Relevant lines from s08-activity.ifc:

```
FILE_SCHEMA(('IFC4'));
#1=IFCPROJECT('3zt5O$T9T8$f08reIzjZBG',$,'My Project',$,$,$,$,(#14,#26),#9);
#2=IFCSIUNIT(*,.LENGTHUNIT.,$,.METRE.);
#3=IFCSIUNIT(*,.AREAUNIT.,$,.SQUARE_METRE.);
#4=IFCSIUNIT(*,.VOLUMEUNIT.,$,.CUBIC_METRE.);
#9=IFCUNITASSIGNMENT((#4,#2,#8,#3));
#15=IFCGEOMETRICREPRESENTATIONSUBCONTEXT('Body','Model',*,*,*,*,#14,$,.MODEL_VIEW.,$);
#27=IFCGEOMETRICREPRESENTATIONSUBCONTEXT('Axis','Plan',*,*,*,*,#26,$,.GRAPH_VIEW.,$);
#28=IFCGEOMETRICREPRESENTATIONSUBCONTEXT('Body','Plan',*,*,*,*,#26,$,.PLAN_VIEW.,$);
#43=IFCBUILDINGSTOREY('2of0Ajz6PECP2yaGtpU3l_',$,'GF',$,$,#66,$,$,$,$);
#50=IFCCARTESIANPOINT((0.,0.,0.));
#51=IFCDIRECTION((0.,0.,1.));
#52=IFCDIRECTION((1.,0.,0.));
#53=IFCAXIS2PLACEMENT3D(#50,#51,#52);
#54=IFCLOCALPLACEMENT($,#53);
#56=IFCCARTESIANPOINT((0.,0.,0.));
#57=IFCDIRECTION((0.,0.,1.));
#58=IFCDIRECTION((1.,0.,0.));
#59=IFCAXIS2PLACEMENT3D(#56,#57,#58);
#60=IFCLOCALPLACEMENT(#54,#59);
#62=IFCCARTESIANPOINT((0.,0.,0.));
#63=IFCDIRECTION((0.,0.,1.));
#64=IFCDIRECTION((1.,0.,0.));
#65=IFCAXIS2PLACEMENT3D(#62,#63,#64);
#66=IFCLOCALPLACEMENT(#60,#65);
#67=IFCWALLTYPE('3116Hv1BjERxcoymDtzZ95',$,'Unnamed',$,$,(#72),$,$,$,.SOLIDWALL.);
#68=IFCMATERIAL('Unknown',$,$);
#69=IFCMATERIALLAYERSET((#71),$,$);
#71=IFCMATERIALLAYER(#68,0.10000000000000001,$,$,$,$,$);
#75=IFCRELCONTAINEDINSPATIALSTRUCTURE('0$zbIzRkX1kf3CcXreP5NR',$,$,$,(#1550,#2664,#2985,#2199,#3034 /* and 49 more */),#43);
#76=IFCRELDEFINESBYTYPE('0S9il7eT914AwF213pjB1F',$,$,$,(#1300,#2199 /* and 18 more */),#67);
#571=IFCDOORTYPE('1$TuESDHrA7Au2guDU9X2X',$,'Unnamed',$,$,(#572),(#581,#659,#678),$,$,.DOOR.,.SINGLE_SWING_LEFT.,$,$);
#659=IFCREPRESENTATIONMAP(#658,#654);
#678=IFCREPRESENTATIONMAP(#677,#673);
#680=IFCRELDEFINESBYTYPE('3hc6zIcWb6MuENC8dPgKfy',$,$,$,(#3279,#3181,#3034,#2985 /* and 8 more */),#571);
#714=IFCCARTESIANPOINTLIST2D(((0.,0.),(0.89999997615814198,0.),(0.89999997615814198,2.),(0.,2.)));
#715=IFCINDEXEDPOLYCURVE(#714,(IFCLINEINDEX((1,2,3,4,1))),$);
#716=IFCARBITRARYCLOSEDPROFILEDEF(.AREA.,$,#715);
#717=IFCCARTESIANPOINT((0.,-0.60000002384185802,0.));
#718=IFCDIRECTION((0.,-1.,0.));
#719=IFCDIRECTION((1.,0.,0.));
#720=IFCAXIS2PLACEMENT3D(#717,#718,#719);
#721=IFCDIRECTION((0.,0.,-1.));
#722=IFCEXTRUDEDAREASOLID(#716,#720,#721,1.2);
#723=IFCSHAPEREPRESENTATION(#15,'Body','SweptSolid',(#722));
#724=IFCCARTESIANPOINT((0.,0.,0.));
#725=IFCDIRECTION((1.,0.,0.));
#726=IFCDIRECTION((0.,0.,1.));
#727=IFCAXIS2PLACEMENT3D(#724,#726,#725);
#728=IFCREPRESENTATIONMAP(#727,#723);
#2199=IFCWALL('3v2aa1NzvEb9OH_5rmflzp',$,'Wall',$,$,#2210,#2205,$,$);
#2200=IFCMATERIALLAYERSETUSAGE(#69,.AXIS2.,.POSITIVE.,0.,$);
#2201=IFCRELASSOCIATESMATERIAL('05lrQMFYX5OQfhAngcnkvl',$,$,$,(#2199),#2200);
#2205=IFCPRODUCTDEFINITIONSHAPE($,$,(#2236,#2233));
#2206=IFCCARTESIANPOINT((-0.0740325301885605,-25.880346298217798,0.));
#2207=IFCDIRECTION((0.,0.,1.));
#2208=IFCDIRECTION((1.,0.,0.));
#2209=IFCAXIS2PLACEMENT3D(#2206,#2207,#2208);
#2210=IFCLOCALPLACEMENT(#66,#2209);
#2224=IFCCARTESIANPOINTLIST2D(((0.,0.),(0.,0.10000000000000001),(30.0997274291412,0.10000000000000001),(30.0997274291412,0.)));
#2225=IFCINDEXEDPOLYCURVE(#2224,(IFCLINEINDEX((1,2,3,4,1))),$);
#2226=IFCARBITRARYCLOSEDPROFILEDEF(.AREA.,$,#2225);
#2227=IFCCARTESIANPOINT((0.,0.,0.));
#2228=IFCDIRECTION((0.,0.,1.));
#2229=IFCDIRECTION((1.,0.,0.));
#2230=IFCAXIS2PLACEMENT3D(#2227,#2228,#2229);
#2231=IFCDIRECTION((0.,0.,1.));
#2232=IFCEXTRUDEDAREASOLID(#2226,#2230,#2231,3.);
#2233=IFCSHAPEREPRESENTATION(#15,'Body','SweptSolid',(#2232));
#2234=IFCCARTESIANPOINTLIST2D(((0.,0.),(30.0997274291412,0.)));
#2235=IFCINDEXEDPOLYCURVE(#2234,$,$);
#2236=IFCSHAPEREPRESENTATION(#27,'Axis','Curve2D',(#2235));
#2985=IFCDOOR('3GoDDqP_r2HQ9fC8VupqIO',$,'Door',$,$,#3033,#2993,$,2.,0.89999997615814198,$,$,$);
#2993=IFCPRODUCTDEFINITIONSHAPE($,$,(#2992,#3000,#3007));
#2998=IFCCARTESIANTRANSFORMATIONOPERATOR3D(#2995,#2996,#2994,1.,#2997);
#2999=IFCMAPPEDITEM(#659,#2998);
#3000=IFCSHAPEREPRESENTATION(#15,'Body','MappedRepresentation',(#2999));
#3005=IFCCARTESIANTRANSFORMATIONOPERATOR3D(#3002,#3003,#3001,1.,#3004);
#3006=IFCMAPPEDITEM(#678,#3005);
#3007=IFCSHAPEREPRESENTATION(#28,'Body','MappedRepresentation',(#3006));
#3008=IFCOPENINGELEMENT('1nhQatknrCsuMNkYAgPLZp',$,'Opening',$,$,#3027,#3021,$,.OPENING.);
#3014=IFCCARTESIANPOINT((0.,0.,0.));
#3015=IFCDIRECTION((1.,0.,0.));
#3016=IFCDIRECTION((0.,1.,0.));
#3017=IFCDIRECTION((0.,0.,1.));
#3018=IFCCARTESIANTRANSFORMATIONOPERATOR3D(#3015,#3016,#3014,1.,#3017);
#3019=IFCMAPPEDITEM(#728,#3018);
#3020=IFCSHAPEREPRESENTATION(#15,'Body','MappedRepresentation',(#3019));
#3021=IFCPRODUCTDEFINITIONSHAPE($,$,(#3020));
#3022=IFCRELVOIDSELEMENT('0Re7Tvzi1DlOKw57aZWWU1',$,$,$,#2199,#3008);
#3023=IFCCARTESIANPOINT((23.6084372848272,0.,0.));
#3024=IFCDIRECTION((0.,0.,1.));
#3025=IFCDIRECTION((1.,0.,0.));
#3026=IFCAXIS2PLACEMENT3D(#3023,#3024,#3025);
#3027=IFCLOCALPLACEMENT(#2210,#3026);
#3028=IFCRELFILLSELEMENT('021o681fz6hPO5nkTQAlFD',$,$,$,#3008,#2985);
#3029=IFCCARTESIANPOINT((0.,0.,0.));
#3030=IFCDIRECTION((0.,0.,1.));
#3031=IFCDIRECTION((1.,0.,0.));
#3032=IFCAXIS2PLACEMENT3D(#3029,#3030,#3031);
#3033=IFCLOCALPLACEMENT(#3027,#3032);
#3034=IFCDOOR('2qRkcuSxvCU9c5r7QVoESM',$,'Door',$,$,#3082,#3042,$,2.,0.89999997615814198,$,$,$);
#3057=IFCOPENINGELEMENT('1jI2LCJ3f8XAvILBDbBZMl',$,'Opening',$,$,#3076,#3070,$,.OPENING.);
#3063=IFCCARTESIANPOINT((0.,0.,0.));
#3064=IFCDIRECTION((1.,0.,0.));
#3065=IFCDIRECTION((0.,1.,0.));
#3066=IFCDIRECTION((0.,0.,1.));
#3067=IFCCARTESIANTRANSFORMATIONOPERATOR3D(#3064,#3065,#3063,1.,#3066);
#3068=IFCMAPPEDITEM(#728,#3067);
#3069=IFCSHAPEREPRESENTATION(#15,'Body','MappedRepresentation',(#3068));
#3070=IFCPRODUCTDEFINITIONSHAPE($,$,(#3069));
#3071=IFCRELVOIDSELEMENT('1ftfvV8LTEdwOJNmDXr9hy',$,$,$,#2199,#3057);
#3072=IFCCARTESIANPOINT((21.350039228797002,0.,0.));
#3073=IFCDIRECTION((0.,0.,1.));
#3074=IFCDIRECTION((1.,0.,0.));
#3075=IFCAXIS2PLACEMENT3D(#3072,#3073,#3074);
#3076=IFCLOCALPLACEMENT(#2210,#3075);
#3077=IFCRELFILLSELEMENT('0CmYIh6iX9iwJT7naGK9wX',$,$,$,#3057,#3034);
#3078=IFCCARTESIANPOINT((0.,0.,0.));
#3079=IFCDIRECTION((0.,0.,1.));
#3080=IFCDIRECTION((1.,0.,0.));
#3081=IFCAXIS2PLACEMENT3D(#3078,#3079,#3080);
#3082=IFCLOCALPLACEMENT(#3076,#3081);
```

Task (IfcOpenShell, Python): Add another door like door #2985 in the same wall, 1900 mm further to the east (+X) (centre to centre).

```python
import ifcopenshell
import ifcopenshell.api.feature
import ifcopenshell.api.geometry
import ifcopenshell.api.root
import ifcopenshell.geom
import ifcopenshell.util.element
import ifcopenshell.util.placement
import ifcopenshell.util.shape
import ifcopenshell.util.unit

model = ifcopenshell.open("s08-activity.ifc")
unit_scale = ifcopenshell.util.unit.calculate_unit_scale(model)
settings = ifcopenshell.geom.settings()


def volume(element):
    """Net volume in cubic metres, openings subtracted."""
    shape = ifcopenshell.geom.create_shape(settings, element)
    return ifcopenshell.util.shape.get_volume(shape.geometry)


door = model.by_guid("3GoDDqP_r2HQ9fC8VupqIO")
opening = door.FillsVoids[0].RelatingOpeningElement
wall = opening.VoidsElements[0].RelatingBuildingElement
before = volume(wall)
shift = ifcopenshell.util.placement.get_local_placement(wall.ObjectPlacement)[:3, 0] * 1.9 / unit_scale

# copy_class copies the void relationship, type, container and properties, but no geometry.
new_opening = ifcopenshell.api.root.copy_class(model, product=opening)
new_opening.Representation = ifcopenshell.util.element.copy_deep(
    model, opening.Representation, exclude=["IfcGeometricRepresentationContext", "IfcRepresentationMap"]
)
new_door = ifcopenshell.api.root.copy_class(model, product=door)
new_door.Representation = ifcopenshell.util.element.copy_deep(
    model, door.Representation, exclude=["IfcGeometricRepresentationContext", "IfcRepresentationMap"]
)
ifcopenshell.api.feature.add_filling(model, opening=new_opening, element=new_door)

for old, new in ((opening, new_opening), (door, new_door)):
    matrix = ifcopenshell.util.placement.get_local_placement(old.ObjectPlacement)
    matrix[:3, 3] += shift
    ifcopenshell.api.geometry.edit_object_placement(model, product=new, matrix=matrix, is_si=False)

after = volume(wall)

print(f"wall volume {before:.3f} -> {after:.3f} m3")

model.write("s08-activity_v2.ifc")
```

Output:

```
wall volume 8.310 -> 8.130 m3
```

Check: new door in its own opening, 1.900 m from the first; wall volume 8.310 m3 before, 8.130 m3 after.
